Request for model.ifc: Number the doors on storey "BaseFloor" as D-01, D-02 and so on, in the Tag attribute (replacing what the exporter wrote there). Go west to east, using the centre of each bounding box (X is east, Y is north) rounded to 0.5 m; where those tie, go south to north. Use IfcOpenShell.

First a look at what the model holds.

```python
import ifcopenshell
import ifcopenshell.util.element
import ifcopenshell.util.placement

model = ifcopenshell.open("model.ifc")
print(model.schema)
storey = next(s for s in model.by_type("IfcBuildingStorey") if s.Name == "BaseFloor")
doors = [e for e in ifcopenshell.util.element.get_decomposition(storey) if e.is_a("IfcDoor")]
for e in sorted(doors, key=lambda e: e.id()):
    origin = ifcopenshell.util.placement.get_local_placement(e.ObjectPlacement)[:3, 3]
    print(e.id(), e.Tag, e.Name, origin.round(2) + 0.0, sep=" | ")
```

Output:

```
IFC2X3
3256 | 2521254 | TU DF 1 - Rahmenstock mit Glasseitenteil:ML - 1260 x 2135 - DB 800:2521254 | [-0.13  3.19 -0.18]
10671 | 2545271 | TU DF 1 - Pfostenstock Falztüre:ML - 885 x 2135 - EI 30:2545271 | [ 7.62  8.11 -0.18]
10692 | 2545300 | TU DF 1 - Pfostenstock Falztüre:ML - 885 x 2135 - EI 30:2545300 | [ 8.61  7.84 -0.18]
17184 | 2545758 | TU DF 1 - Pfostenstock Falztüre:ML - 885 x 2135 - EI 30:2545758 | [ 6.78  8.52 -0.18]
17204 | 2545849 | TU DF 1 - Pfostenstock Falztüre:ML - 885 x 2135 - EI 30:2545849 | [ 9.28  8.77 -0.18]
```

```python
import ifcopenshell
import ifcopenshell.geom
import ifcopenshell.util.element
import ifcopenshell.util.shape

model = ifcopenshell.open("model.ifc")
settings = ifcopenshell.geom.settings()
settings.set("use-world-coords", True)


def centre(element):
    shape = ifcopenshell.geom.create_shape(settings, element)
    return ifcopenshell.util.shape.get_bbox_centroid(shape.geometry)


storey = next(s for s in model.by_type("IfcBuildingStorey") if s.Name == "BaseFloor")
doors = [e for e in ifcopenshell.util.element.get_decomposition(storey) if e.is_a("IfcDoor")]

# Insertion points can sit at a corner or the storey origin, so sort by the geometry (in metres).
centres = {e: centre(e) for e in doors}
doors.sort(key=lambda e: (round(centres[e][0] / 0.5), centres[e][1]))

for i, e in enumerate(doors, start=1):
    number = f"D-{i:02d}"
    e.Tag = number
    print(e.id(), number)

model.write("model_updated.ifc")
```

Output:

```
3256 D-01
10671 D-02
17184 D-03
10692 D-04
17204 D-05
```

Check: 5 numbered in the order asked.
